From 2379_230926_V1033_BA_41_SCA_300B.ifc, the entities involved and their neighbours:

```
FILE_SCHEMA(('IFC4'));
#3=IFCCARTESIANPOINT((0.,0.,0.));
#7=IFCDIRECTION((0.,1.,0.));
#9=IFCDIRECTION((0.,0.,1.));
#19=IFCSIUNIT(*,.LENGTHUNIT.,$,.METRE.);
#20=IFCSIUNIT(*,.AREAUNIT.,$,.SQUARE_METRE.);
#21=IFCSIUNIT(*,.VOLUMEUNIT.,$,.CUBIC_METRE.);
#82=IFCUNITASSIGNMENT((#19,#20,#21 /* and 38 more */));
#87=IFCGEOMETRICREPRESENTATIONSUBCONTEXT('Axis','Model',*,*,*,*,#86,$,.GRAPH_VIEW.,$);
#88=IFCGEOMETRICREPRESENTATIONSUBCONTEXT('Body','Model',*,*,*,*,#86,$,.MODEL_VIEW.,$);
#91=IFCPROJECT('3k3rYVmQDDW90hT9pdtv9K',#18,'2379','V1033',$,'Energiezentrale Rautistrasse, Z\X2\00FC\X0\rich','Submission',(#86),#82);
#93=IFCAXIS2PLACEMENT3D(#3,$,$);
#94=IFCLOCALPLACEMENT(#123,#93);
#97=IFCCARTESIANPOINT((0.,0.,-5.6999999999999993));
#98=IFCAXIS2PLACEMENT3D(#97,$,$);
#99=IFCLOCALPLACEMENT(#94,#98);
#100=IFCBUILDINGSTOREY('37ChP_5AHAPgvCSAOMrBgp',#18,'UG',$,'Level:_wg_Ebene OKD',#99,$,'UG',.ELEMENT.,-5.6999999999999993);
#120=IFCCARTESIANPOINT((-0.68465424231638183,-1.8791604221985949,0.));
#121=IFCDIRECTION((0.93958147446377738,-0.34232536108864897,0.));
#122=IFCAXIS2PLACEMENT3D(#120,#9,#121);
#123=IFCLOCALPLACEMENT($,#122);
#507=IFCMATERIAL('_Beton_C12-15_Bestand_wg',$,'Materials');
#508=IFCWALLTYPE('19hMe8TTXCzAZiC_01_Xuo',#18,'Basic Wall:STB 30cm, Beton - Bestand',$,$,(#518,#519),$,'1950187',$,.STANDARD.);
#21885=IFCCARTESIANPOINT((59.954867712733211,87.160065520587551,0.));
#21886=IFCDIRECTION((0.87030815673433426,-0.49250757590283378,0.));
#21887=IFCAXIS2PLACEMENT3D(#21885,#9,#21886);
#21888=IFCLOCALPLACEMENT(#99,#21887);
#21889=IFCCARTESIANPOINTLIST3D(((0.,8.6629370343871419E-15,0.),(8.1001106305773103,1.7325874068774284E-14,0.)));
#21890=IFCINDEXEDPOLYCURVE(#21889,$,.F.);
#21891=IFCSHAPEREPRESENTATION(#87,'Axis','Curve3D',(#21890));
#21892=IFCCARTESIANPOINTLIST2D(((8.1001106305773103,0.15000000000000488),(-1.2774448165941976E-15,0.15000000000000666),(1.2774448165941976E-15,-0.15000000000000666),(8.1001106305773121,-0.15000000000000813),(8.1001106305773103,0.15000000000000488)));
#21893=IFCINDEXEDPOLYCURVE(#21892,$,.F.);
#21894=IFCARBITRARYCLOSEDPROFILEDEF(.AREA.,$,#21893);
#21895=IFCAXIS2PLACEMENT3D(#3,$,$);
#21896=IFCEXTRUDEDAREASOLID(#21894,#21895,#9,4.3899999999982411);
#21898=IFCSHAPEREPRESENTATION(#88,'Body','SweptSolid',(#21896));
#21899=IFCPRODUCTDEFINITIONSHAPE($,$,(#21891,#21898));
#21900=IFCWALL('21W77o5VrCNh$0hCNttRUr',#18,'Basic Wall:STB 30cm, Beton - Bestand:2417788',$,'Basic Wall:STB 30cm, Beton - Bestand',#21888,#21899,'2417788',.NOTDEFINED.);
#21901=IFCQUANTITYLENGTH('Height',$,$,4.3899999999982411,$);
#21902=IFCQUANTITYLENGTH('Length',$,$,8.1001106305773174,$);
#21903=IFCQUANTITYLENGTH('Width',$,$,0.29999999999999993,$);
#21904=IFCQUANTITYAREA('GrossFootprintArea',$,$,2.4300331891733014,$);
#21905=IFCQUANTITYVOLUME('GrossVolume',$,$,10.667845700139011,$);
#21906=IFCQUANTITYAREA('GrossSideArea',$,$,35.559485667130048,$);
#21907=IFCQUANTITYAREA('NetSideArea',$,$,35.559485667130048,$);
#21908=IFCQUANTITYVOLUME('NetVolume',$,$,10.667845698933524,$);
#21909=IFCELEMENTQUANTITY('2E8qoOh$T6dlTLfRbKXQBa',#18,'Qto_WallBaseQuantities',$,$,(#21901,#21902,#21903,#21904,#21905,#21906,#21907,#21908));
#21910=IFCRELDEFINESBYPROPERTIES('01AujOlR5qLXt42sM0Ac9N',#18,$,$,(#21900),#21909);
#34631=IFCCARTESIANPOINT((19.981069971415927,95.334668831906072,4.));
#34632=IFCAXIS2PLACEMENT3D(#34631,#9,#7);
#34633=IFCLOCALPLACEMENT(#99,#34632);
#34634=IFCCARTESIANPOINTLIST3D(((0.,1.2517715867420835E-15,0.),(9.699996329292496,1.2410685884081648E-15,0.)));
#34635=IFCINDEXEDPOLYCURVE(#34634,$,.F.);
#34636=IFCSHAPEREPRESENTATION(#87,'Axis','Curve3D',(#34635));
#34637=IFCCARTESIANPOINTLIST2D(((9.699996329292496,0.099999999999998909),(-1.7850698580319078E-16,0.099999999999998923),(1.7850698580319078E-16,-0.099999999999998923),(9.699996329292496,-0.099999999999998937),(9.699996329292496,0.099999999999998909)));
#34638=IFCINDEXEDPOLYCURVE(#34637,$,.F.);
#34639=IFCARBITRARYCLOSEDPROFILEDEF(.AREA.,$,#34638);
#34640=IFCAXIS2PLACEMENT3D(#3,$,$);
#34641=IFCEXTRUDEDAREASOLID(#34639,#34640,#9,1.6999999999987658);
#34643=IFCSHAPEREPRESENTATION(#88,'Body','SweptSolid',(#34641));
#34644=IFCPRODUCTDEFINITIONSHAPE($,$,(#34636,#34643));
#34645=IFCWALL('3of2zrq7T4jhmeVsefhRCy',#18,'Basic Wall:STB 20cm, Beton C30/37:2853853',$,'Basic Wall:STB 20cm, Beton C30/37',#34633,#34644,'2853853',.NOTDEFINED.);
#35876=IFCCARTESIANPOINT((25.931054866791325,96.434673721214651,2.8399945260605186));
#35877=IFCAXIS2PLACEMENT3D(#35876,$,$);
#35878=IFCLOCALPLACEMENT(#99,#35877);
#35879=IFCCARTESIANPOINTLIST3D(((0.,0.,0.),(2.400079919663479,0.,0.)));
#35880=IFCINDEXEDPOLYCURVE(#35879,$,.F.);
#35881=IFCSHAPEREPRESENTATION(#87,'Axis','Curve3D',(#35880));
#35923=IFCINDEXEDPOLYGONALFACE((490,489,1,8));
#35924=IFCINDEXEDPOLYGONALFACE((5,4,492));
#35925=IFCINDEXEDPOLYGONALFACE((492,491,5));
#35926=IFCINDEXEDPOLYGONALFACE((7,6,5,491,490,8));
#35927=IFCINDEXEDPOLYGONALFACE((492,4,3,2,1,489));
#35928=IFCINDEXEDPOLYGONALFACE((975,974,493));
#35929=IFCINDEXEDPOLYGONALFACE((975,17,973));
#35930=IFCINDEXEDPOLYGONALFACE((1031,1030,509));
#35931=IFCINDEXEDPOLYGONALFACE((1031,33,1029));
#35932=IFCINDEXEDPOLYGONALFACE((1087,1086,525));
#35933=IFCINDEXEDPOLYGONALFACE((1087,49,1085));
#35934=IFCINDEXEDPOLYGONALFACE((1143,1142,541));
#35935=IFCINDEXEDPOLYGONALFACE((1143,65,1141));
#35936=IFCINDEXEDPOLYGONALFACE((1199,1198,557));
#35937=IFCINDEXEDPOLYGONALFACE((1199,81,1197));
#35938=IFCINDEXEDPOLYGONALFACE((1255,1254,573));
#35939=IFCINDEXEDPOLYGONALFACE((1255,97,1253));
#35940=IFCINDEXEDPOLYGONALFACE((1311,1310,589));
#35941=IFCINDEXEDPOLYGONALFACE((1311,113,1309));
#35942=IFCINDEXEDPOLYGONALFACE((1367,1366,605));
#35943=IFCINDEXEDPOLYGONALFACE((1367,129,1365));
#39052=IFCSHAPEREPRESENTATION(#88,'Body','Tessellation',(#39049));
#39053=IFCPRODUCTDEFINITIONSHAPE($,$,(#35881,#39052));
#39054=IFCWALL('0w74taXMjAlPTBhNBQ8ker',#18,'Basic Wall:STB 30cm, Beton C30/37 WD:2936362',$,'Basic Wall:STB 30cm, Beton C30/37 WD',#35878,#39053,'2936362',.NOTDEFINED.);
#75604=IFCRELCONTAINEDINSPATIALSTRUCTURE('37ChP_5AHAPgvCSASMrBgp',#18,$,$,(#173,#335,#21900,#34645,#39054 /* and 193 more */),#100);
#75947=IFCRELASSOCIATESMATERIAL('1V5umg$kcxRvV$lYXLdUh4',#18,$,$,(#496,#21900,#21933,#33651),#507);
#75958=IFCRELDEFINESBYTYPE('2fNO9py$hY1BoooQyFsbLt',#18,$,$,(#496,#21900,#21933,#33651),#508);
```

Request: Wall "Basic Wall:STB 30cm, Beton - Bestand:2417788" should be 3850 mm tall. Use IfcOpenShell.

```python
import ifcopenshell
import ifcopenshell.api.pset
import ifcopenshell.geom
import ifcopenshell.util.element
import ifcopenshell.util.representation
import ifcopenshell.util.shape
import ifcopenshell.util.unit

model = ifcopenshell.open("2379_230926_V1033_BA_41_SCA_300B.ifc")
unit_scale = ifcopenshell.util.unit.calculate_unit_scale(model)
area_scale = ifcopenshell.util.unit.calculate_unit_scale(model, "AREAUNIT")
volume_scale = ifcopenshell.util.unit.calculate_unit_scale(model, "VOLUMEUNIT")
settings = ifcopenshell.geom.settings()


def volume(element):
    """Net volume in cubic metres, openings subtracted."""
    shape = ifcopenshell.geom.create_shape(settings, element)
    return ifcopenshell.util.shape.get_volume(shape.geometry)


wall = model.by_guid("21W77o5VrCNh$0hCNttRUr")
before = volume(wall)

body = ifcopenshell.util.representation.get_representation(wall, "Model", "Body")
solid = body.Items[0]
old_height = solid.Depth
solid.Depth = 3.85
after = volume(wall)
thickness = 0.3  # wall thickness in metres

# Update the stored height, areas and volumes.
qto = model.by_id(ifcopenshell.util.element.get_pset(wall, "Qto_WallBaseQuantities", should_inherit=False)["id"])
ifcopenshell.api.pset.edit_qto(model, qto=qto, properties={
    "Height": solid.Depth,
    "GrossVolume": ifcopenshell.util.element.get_pset(wall, "Qto_WallBaseQuantities", "GrossVolume") * solid.Depth / old_height,
    "GrossSideArea": ifcopenshell.util.element.get_pset(wall, "Qto_WallBaseQuantities", "GrossSideArea") * solid.Depth / old_height,
    "NetSideArea": after / thickness / area_scale,
    "NetVolume": after / volume_scale,
})

print(f"height {old_height:g} -> {solid.Depth:g}, volume {before:.3f} -> {after:.3f} m3")

model.write("2379_230926_V1033_BA_41_SCA_300B-out.ifc")
```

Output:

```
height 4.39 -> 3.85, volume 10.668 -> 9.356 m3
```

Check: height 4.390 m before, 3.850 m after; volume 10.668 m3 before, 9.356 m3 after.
